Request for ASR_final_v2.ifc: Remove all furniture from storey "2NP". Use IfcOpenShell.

First a look at what the model holds.

```python
import ifcopenshell
import ifcopenshell.util.element

model = ifcopenshell.open("ASR_final_v2.ifc")
print(model.schema)
storey = next(s for s in model.by_type("IfcBuildingStorey") if s.Name == "2NP")
furniture = [e for e in ifcopenshell.util.element.get_decomposition(storey) if e.is_a("IfcFurnishingElement")]
seen = {}
for e in furniture:
    element_type = ifcopenshell.util.element.get_type(e)
    name = element_type.Name if element_type not in (None, e) else None
    seen[name] = seen.get(name, 0) + 1
for name, count in sorted(seen.items(), key=str):
    print(count, "x", name)
```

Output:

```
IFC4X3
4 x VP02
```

```python
import ifcopenshell
import ifcopenshell.api.root
import ifcopenshell.util.element

model = ifcopenshell.open("ASR_final_v2.ifc")

storey = next(s for s in model.by_type("IfcBuildingStorey") if s.Name == "2NP")
furniture = [e for e in ifcopenshell.util.element.get_decomposition(storey) if e.is_a("IfcFurnishingElement")]

for e in furniture:
    ifcopenshell.api.root.remove_product(model, product=e)
print(len(furniture), "removed")

model.write("ASR_final_v2_rev.ifc")
```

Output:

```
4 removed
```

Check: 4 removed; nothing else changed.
